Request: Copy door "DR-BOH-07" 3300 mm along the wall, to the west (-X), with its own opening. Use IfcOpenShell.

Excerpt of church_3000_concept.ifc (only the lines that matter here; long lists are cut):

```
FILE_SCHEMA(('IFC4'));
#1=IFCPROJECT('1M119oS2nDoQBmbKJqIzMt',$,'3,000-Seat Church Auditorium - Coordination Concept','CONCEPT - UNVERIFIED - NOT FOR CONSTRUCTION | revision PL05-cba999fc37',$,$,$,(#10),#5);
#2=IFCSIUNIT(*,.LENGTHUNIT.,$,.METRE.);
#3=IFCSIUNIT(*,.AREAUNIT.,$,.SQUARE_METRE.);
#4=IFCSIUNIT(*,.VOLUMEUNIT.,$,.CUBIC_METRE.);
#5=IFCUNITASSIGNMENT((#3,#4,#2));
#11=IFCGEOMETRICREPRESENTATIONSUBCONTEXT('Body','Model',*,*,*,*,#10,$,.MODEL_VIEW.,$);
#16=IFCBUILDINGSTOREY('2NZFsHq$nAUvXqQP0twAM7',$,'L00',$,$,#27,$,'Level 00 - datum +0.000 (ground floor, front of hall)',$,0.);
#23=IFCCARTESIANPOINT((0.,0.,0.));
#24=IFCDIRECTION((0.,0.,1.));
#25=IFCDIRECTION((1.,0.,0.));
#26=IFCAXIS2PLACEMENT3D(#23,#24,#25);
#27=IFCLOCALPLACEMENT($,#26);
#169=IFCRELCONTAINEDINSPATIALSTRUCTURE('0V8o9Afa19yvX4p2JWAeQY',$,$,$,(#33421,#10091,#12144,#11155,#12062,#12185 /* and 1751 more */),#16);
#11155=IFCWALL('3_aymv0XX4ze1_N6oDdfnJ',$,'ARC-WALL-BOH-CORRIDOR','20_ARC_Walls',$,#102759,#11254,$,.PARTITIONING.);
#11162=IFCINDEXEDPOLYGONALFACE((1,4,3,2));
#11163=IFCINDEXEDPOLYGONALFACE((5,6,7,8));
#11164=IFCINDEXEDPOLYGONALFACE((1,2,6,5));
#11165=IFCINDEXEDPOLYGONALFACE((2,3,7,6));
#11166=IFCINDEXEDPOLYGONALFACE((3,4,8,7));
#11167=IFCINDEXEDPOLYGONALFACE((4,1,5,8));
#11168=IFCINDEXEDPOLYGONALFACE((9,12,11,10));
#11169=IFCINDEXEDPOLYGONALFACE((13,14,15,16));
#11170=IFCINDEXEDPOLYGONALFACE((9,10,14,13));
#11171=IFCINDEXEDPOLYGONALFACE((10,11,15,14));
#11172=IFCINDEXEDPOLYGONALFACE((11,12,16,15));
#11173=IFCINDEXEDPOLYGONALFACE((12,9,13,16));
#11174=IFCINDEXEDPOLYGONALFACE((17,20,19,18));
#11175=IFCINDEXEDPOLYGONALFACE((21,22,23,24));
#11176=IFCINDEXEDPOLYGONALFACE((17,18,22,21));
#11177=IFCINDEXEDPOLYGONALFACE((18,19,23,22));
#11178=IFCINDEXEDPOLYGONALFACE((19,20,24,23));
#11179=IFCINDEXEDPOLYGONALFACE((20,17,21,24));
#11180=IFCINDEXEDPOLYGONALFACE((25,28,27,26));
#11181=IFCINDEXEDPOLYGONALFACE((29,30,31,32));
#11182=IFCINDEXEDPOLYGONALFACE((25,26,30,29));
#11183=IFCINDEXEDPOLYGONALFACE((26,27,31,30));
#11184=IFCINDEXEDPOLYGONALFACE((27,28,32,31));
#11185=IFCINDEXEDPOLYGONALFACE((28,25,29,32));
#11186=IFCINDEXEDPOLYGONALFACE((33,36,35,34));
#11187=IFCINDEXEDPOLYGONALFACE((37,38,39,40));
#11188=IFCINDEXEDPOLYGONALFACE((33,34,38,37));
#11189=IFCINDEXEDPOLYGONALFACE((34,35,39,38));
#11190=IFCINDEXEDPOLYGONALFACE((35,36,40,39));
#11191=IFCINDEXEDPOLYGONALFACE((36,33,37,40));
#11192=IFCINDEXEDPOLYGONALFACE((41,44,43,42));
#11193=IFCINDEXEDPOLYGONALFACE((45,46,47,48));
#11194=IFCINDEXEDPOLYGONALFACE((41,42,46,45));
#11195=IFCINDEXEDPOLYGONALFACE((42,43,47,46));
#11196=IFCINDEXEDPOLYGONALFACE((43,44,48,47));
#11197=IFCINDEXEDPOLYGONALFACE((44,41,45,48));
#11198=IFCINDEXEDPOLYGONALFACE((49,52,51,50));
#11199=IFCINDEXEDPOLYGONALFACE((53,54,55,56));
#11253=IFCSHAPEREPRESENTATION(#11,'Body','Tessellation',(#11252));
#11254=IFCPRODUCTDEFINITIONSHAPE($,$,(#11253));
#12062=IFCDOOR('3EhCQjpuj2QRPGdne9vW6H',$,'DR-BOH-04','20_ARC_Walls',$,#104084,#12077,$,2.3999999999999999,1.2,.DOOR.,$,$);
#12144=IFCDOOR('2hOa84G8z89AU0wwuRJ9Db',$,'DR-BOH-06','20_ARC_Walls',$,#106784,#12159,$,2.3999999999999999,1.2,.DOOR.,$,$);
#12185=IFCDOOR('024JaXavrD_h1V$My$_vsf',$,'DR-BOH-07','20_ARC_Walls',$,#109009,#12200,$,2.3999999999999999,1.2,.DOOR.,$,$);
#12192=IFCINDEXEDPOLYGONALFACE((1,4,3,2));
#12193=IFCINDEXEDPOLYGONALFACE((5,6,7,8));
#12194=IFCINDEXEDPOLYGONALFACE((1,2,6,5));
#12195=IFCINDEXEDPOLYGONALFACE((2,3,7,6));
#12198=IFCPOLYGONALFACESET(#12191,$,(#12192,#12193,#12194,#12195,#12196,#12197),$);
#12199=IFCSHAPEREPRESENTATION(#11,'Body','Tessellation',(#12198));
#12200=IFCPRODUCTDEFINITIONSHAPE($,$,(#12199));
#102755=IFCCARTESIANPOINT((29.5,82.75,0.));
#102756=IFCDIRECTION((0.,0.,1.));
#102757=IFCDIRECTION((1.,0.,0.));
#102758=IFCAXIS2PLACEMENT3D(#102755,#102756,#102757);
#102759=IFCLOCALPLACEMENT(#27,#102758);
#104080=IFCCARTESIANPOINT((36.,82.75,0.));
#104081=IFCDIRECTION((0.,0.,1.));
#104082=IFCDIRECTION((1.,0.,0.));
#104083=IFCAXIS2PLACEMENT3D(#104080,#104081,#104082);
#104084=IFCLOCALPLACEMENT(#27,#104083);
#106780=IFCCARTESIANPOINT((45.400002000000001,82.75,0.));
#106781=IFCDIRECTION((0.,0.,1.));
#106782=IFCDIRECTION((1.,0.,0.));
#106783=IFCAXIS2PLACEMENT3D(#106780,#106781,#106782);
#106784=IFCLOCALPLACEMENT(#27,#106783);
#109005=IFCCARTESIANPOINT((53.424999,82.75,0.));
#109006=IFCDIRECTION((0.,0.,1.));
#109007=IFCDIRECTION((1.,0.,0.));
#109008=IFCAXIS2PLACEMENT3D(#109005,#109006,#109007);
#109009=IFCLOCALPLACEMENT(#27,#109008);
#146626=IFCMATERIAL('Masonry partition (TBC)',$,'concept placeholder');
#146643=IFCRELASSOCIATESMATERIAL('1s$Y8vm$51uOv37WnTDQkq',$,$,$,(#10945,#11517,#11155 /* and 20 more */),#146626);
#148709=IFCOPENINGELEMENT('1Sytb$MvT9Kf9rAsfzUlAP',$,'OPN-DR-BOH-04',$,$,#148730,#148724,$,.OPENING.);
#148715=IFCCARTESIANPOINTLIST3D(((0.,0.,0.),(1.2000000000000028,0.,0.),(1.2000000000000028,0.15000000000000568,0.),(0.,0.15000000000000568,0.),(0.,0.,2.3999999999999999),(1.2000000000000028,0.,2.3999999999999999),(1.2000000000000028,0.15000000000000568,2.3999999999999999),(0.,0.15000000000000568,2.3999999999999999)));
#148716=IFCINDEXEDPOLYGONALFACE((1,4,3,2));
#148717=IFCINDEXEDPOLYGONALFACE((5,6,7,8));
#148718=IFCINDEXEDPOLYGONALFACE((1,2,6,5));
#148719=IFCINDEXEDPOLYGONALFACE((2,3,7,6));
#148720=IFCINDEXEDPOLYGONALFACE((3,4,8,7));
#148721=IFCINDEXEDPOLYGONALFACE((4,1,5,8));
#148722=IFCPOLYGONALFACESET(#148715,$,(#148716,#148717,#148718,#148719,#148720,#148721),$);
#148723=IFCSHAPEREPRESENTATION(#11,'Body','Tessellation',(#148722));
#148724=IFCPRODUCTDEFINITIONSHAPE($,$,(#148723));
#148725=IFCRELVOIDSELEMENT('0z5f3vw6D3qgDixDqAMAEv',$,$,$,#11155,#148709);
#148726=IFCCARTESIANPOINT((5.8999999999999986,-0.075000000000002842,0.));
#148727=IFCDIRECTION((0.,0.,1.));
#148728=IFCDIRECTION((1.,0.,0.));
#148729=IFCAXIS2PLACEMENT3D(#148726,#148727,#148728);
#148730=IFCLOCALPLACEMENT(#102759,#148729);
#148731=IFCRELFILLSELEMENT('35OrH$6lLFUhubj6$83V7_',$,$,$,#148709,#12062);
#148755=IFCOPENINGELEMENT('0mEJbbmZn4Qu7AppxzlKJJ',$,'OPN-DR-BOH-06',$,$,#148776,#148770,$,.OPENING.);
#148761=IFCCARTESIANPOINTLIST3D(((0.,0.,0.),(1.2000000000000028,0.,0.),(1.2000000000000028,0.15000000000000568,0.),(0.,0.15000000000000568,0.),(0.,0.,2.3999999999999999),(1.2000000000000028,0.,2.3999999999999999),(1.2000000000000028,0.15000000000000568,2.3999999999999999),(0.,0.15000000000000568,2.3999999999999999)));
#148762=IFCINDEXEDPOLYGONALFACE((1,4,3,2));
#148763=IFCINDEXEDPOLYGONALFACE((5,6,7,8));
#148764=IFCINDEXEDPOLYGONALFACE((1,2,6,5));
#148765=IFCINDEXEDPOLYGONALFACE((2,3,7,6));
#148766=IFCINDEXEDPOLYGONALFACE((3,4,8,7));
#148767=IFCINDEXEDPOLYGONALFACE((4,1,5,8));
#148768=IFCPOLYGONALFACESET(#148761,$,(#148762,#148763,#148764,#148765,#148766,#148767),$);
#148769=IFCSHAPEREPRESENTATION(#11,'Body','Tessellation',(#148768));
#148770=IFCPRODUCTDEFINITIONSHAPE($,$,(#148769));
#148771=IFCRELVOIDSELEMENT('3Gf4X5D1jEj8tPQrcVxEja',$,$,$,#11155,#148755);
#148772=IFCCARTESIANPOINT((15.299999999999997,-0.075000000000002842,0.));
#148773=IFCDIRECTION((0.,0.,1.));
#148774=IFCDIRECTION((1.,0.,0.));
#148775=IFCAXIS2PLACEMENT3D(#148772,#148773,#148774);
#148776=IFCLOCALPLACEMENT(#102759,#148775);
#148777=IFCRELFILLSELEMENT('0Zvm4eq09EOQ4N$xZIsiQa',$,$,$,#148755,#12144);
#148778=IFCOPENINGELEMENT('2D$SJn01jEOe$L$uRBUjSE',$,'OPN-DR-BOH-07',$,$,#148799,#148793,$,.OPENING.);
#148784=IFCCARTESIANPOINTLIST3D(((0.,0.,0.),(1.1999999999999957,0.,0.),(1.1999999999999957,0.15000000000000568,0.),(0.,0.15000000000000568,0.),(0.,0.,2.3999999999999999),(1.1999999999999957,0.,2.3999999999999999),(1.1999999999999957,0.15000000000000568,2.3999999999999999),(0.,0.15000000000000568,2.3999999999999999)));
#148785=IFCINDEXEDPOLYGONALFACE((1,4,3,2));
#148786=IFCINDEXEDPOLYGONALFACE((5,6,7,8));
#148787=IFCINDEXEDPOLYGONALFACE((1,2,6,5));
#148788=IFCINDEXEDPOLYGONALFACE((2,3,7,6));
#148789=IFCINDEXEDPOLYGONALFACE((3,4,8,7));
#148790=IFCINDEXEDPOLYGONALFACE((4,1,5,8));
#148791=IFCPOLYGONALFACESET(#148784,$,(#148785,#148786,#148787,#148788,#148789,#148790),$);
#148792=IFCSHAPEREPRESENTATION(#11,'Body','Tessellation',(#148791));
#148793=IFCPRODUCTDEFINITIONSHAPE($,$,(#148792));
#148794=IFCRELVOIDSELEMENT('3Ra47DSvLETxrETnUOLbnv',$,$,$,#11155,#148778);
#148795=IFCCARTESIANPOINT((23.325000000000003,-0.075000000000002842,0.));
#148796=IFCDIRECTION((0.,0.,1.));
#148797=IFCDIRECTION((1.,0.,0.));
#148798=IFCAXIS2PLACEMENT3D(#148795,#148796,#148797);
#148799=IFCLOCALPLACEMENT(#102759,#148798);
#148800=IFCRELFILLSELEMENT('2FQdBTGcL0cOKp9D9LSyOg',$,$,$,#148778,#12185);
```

```python
import ifcopenshell
import ifcopenshell.api.feature
import ifcopenshell.api.geometry
import ifcopenshell.api.root
import ifcopenshell.geom
import ifcopenshell.util.element
import ifcopenshell.util.placement
import ifcopenshell.util.shape
import ifcopenshell.util.unit

model = ifcopenshell.open("church_3000_concept.ifc")
unit_scale = ifcopenshell.util.unit.calculate_unit_scale(model)
settings = ifcopenshell.geom.settings()


def volume(element):
    """Net volume in cubic metres, openings subtracted."""
    shape = ifcopenshell.geom.create_shape(settings, element)
    return ifcopenshell.util.shape.get_volume(shape.geometry)


door = model.by_guid("024JaXavrD_h1V$My$_vsf")
opening = door.FillsVoids[0].RelatingOpeningElement
wall = opening.VoidsElements[0].RelatingBuildingElement
before = volume(wall)
shift = ifcopenshell.util.placement.get_local_placement(wall.ObjectPlacement)[:3, 0] * -3.3 / unit_scale

# copy_class copies the void relationship, type, container and properties, but no geometry.
new_opening = ifcopenshell.api.root.copy_class(model, product=opening)
new_opening.Representation = ifcopenshell.util.element.copy_deep(
    model, opening.Representation, exclude=["IfcGeometricRepresentationContext", "IfcRepresentationMap"]
)
new_door = ifcopenshell.api.root.copy_class(model, product=door)
new_door.Representation = ifcopenshell.util.element.copy_deep(
    model, door.Representation, exclude=["IfcGeometricRepresentationContext", "IfcRepresentationMap"]
)
ifcopenshell.api.feature.add_filling(model, opening=new_opening, element=new_door)

for old, new in ((opening, new_opening), (door, new_door)):
    matrix = ifcopenshell.util.placement.get_local_placement(old.ObjectPlacement)
    matrix[:3, 3] += shift
    ifcopenshell.api.geometry.edit_object_placement(model, product=new, matrix=matrix, is_si=False)

after = volume(wall)

print(f"wall volume {before:.3f} -> {after:.3f} m3")

model.write("church_3000_concept_edited.ifc")
```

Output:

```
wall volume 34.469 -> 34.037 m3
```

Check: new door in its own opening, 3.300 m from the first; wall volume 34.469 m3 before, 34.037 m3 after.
